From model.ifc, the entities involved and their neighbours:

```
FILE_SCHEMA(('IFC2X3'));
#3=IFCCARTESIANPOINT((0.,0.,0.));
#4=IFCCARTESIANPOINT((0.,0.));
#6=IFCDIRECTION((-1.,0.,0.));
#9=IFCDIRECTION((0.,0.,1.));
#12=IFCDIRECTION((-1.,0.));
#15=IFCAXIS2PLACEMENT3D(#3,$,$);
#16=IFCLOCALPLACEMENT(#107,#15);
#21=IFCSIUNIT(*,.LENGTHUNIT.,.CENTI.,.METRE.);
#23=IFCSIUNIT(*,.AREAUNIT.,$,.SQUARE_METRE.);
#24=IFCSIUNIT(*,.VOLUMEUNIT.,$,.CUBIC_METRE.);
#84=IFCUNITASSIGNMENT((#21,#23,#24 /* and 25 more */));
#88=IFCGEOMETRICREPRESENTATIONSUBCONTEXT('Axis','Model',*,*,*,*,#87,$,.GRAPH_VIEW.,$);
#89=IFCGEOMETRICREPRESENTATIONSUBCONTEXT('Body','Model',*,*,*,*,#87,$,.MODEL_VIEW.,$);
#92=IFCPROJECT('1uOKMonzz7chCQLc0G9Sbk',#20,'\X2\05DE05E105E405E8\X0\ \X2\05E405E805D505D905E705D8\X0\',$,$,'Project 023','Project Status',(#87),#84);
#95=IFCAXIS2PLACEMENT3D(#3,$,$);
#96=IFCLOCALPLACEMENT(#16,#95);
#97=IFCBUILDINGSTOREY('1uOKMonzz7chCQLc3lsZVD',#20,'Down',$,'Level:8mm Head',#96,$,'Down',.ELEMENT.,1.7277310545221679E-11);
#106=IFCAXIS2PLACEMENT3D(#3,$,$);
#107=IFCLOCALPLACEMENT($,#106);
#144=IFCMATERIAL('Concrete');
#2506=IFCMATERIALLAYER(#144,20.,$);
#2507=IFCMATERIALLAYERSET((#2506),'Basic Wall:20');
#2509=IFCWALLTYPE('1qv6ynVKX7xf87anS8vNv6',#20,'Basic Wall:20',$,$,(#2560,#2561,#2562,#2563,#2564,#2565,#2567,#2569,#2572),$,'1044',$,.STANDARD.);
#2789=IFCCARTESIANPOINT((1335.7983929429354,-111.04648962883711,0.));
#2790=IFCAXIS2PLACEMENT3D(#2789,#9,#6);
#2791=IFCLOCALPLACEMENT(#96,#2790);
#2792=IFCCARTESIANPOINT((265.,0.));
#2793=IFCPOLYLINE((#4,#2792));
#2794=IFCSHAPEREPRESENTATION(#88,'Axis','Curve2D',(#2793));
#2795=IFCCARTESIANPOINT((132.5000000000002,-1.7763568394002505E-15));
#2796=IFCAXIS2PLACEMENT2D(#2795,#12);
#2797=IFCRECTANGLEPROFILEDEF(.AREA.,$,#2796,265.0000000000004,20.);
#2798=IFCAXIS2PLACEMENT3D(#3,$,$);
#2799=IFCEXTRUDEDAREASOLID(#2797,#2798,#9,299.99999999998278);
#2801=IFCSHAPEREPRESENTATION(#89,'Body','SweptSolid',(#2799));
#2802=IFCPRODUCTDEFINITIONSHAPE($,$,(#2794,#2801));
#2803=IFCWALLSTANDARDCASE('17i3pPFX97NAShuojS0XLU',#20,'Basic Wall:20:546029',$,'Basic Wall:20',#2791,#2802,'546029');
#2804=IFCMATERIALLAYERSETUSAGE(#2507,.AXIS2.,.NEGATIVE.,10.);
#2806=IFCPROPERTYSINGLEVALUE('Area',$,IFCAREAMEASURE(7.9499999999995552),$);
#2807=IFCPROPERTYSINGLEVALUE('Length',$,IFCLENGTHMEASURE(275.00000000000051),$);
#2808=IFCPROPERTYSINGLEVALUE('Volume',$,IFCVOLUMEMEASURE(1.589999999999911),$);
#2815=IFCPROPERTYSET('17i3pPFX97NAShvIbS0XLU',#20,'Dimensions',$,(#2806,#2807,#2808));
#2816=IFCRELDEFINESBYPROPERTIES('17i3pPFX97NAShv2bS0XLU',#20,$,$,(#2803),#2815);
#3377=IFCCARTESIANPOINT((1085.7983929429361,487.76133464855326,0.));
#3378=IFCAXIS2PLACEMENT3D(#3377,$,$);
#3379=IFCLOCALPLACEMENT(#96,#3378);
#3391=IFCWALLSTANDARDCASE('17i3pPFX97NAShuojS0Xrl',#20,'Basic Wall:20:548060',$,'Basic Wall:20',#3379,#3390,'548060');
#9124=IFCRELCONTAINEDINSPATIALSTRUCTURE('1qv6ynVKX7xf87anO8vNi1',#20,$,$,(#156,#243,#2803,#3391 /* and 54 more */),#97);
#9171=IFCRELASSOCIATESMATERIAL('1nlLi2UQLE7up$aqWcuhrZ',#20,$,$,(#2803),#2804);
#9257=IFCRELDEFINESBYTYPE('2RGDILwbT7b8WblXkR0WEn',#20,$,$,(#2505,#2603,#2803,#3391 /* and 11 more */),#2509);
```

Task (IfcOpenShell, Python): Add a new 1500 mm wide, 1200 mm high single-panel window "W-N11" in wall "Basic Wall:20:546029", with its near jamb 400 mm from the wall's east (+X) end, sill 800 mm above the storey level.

```python
import numpy as np
import ifcopenshell
import ifcopenshell.api.feature
import ifcopenshell.api.geometry
import ifcopenshell.api.pset
import ifcopenshell.api.root
import ifcopenshell.api.spatial
import ifcopenshell.api.type
import ifcopenshell.geom
import ifcopenshell.util.element
import ifcopenshell.util.placement
import ifcopenshell.util.representation
import ifcopenshell.util.shape
import ifcopenshell.util.unit

model = ifcopenshell.open("model.ifc")
unit_scale = ifcopenshell.util.unit.calculate_unit_scale(model)
area_scale = ifcopenshell.util.unit.calculate_unit_scale(model, "AREAUNIT")
volume_scale = ifcopenshell.util.unit.calculate_unit_scale(model, "VOLUMEUNIT")
settings = ifcopenshell.geom.settings()


def volume(element):
    """Net volume in cubic metres, openings subtracted."""
    shape = ifcopenshell.geom.create_shape(settings, element)
    return ifcopenshell.util.shape.get_volume(shape.geometry)


wall = model.by_guid("17i3pPFX97NAShuojS0XLU")
storey = ifcopenshell.util.element.get_container(wall, ifc_class="IfcBuildingStorey")
context = ifcopenshell.util.representation.get_context(model, "Model", "Body", "MODEL_VIEW")
before = volume(wall)

width, height, from_end, sill = 1.5, 1.2, 0.4, 0.8  # metres

# The wall runs along its own X axis, and the end named is its -X end.
wall_shape = ifcopenshell.geom.create_shape(settings, wall)
x, y, z = ifcopenshell.util.shape.get_vertices(wall_shape.geometry).T
start = x.min() + from_end
face, thickness = float(y.min()), float(y.max() - y.min())
wall_matrix = ifcopenshell.util.placement.get_local_placement(wall.ObjectPlacement)
level = ifcopenshell.util.placement.get_local_placement(storey.ObjectPlacement)[2, 3]


def in_wall(x, y):
    """Placement at x, y metres in the wall's axes, at sill height."""
    matrix = wall_matrix.copy()
    matrix[:, 3] = wall_matrix @ np.array([x / unit_scale, y / unit_scale, 0.0, 1.0])
    matrix[2, 3] = level + sill / unit_scale
    return matrix


# Opening: a box that overshoots both wall faces by 50 mm.
opening = ifcopenshell.api.root.create_entity(model, ifc_class="IfcOpeningElement")
box = ifcopenshell.api.geometry.add_wall_representation(
    model, context=context, length=width, height=height, thickness=thickness + 0.1
)
ifcopenshell.api.geometry.assign_representation(model, product=opening, representation=box)
ifcopenshell.api.geometry.edit_object_placement(model, product=opening, matrix=in_wall(start, face - 0.05), is_si=False)
ifcopenshell.api.feature.add_feature(model, feature=opening, element=wall)

window = ifcopenshell.api.root.create_entity(model, ifc_class="IfcWindow", name="W-N11")
window.OverallWidth, window.OverallHeight = width / unit_scale, height / unit_scale
body = ifcopenshell.api.geometry.add_window_representation(
    model,
    context=context,
    overall_width=window.OverallWidth,
    overall_height=window.OverallHeight,
    partition_type="SINGLE_PANEL",
)
ifcopenshell.api.geometry.assign_representation(model, product=window, representation=body)
ifcopenshell.api.spatial.assign_container(model, products=[window], relating_structure=storey)
fills = ifcopenshell.api.feature.add_filling(model, opening=opening, element=window)
fills.OwnerHistory = window.OwnerHistory  # required in IFC2X3

# IFC2X3 keeps the operation on the window style.
style = ifcopenshell.api.root.create_entity(model, ifc_class="IfcWindowStyle", name="W-N11")
style.OperationType, style.ConstructionType = "SINGLE_PANEL", "NOTDEFINED"
style.ParameterTakesPrecedence = style.Sizeable = False
ifcopenshell.api.type.assign_type(model, related_objects=[window], relating_type=style)

# Centre the window in the wall's thickness.
ifcopenshell.api.geometry.edit_object_placement(model, product=window, matrix=in_wall(start, face), is_si=False)
window_shape = ifcopenshell.geom.create_shape(settings, window)
depth = ifcopenshell.util.shape.get_vertices(window_shape.geometry)[:, 1]
offset = face + thickness / 2 - (depth.min() + depth.max()) / 2
ifcopenshell.api.geometry.edit_object_placement(model, product=window, matrix=in_wall(start, offset), is_si=False)

after = volume(wall)

# Update the wall's stored quantities.
pset = model.by_id(ifcopenshell.util.element.get_pset(wall, "Dimensions", should_inherit=False)["id"])
ifcopenshell.api.pset.edit_pset(model, pset=pset, properties={
    "Area": model.create_entity("IfcAreaMeasure", after / thickness / area_scale),
    "Volume": model.create_entity("IfcVolumeMeasure", after / volume_scale),
})

print(f"wall volume {before:.3f} -> {after:.3f} m3")

model.write("model_updated.ifc")
```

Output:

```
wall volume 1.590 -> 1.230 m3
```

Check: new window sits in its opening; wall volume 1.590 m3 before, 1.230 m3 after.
